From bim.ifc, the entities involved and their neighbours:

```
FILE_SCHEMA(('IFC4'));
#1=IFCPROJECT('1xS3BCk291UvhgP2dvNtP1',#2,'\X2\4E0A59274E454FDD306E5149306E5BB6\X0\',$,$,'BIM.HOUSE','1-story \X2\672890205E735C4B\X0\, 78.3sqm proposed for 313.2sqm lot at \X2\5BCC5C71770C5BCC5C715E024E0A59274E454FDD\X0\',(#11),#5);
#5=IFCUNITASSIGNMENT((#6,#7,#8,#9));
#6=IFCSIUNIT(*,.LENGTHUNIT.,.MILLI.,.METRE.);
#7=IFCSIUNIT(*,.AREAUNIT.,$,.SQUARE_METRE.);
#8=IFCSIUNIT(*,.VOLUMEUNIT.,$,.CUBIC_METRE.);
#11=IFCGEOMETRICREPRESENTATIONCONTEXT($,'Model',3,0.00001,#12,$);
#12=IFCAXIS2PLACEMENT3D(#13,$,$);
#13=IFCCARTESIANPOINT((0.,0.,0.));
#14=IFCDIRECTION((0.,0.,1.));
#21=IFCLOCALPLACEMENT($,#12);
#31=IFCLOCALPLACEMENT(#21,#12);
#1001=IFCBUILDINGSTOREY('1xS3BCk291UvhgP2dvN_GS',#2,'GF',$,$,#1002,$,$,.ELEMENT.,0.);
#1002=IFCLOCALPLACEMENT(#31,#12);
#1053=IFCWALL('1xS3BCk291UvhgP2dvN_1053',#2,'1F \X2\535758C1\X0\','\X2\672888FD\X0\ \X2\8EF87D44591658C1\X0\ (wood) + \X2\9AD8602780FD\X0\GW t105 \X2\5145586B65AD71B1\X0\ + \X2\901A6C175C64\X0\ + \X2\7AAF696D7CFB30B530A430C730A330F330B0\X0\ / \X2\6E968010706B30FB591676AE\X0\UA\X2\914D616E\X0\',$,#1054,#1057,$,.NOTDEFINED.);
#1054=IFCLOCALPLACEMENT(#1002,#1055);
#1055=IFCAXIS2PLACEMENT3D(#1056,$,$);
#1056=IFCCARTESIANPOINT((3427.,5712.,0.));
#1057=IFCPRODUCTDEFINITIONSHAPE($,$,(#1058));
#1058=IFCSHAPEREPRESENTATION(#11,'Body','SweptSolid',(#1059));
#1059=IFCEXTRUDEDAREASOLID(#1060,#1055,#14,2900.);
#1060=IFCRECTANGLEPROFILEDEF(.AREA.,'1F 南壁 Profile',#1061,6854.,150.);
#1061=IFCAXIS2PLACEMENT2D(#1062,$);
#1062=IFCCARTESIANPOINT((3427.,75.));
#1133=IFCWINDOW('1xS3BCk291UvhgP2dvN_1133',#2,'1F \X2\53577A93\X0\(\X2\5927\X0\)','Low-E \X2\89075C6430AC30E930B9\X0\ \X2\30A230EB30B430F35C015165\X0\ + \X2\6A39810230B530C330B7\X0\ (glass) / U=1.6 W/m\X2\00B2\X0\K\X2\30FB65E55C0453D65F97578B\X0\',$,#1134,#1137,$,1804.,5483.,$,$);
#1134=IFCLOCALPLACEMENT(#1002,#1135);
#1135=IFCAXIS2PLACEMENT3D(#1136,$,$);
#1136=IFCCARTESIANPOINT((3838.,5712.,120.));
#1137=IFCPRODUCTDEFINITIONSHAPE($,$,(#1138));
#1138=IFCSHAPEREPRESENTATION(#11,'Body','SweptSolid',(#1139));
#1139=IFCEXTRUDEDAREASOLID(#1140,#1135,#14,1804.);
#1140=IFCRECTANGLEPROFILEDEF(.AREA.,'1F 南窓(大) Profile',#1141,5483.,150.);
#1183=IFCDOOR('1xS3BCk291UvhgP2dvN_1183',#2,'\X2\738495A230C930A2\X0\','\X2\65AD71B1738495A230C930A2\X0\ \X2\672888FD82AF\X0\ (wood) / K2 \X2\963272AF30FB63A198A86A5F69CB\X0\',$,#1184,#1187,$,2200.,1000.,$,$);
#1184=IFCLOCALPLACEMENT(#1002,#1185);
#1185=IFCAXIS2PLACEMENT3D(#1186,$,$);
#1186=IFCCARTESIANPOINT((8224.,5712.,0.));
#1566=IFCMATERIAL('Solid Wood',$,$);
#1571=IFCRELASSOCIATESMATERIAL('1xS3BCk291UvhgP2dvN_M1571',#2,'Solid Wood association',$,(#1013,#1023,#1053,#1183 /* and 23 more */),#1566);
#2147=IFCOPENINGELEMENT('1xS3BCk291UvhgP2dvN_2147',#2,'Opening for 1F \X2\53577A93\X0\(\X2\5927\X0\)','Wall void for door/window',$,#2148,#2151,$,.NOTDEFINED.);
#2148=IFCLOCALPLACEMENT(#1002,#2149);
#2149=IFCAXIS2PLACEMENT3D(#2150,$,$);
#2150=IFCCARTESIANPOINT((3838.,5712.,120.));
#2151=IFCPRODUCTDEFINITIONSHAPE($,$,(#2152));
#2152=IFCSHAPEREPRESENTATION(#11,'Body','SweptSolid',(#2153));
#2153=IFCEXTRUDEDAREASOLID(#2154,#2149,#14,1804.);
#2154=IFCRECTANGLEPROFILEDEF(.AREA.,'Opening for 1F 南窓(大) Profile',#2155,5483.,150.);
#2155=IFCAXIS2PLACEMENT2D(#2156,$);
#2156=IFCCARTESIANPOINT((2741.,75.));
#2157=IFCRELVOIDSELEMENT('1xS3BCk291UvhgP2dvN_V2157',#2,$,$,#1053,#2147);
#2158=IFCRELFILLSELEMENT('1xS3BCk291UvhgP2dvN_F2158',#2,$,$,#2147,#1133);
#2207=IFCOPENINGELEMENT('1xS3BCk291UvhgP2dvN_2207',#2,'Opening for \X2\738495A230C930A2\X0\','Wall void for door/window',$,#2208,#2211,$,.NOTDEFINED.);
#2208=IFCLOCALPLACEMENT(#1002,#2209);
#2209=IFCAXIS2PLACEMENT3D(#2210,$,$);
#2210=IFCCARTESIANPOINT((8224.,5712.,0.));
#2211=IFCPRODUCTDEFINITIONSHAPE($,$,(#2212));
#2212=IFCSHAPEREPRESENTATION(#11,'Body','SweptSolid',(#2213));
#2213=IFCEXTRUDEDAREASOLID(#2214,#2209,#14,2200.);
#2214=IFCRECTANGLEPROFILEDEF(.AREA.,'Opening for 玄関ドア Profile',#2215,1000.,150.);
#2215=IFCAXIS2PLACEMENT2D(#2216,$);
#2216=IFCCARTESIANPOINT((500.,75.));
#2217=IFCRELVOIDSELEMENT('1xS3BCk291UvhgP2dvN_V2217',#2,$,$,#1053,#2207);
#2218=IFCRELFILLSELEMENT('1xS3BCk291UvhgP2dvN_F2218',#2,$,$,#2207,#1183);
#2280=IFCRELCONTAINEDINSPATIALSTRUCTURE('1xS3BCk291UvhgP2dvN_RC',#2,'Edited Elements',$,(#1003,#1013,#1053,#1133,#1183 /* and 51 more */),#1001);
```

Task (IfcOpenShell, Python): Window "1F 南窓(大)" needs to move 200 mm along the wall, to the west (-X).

```python
import ifcopenshell
import ifcopenshell.api.geometry
import ifcopenshell.util.placement
import ifcopenshell.util.unit

model = ifcopenshell.open("bim.ifc")
unit_scale = ifcopenshell.util.unit.calculate_unit_scale(model)

window = model.by_id(1133)
opening = window.FillsVoids[0].RelatingOpeningElement
wall = opening.VoidsElements[0].RelatingBuildingElement

wall_matrix = ifcopenshell.util.placement.get_local_placement(wall.ObjectPlacement)
shift = wall_matrix[:3, 0] * -0.2 / unit_scale
before = ifcopenshell.util.placement.get_local_placement(window.ObjectPlacement)[:3, 3].copy()

# The window is not placed relative to its opening, so move both.
for product in (opening, window):
    matrix = ifcopenshell.util.placement.get_local_placement(product.ObjectPlacement)
    matrix[:3, 3] += shift
    ifcopenshell.api.geometry.edit_object_placement(model, product=product, matrix=matrix, is_si=False)

after = ifcopenshell.util.placement.get_local_placement(window.ObjectPlacement)[:3, 3]
print("window moved by", (after - before).round(3) + 0.0)

model.write("bim_rev.ifc")
```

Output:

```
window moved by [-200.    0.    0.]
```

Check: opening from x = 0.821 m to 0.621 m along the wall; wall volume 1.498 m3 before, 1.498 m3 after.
